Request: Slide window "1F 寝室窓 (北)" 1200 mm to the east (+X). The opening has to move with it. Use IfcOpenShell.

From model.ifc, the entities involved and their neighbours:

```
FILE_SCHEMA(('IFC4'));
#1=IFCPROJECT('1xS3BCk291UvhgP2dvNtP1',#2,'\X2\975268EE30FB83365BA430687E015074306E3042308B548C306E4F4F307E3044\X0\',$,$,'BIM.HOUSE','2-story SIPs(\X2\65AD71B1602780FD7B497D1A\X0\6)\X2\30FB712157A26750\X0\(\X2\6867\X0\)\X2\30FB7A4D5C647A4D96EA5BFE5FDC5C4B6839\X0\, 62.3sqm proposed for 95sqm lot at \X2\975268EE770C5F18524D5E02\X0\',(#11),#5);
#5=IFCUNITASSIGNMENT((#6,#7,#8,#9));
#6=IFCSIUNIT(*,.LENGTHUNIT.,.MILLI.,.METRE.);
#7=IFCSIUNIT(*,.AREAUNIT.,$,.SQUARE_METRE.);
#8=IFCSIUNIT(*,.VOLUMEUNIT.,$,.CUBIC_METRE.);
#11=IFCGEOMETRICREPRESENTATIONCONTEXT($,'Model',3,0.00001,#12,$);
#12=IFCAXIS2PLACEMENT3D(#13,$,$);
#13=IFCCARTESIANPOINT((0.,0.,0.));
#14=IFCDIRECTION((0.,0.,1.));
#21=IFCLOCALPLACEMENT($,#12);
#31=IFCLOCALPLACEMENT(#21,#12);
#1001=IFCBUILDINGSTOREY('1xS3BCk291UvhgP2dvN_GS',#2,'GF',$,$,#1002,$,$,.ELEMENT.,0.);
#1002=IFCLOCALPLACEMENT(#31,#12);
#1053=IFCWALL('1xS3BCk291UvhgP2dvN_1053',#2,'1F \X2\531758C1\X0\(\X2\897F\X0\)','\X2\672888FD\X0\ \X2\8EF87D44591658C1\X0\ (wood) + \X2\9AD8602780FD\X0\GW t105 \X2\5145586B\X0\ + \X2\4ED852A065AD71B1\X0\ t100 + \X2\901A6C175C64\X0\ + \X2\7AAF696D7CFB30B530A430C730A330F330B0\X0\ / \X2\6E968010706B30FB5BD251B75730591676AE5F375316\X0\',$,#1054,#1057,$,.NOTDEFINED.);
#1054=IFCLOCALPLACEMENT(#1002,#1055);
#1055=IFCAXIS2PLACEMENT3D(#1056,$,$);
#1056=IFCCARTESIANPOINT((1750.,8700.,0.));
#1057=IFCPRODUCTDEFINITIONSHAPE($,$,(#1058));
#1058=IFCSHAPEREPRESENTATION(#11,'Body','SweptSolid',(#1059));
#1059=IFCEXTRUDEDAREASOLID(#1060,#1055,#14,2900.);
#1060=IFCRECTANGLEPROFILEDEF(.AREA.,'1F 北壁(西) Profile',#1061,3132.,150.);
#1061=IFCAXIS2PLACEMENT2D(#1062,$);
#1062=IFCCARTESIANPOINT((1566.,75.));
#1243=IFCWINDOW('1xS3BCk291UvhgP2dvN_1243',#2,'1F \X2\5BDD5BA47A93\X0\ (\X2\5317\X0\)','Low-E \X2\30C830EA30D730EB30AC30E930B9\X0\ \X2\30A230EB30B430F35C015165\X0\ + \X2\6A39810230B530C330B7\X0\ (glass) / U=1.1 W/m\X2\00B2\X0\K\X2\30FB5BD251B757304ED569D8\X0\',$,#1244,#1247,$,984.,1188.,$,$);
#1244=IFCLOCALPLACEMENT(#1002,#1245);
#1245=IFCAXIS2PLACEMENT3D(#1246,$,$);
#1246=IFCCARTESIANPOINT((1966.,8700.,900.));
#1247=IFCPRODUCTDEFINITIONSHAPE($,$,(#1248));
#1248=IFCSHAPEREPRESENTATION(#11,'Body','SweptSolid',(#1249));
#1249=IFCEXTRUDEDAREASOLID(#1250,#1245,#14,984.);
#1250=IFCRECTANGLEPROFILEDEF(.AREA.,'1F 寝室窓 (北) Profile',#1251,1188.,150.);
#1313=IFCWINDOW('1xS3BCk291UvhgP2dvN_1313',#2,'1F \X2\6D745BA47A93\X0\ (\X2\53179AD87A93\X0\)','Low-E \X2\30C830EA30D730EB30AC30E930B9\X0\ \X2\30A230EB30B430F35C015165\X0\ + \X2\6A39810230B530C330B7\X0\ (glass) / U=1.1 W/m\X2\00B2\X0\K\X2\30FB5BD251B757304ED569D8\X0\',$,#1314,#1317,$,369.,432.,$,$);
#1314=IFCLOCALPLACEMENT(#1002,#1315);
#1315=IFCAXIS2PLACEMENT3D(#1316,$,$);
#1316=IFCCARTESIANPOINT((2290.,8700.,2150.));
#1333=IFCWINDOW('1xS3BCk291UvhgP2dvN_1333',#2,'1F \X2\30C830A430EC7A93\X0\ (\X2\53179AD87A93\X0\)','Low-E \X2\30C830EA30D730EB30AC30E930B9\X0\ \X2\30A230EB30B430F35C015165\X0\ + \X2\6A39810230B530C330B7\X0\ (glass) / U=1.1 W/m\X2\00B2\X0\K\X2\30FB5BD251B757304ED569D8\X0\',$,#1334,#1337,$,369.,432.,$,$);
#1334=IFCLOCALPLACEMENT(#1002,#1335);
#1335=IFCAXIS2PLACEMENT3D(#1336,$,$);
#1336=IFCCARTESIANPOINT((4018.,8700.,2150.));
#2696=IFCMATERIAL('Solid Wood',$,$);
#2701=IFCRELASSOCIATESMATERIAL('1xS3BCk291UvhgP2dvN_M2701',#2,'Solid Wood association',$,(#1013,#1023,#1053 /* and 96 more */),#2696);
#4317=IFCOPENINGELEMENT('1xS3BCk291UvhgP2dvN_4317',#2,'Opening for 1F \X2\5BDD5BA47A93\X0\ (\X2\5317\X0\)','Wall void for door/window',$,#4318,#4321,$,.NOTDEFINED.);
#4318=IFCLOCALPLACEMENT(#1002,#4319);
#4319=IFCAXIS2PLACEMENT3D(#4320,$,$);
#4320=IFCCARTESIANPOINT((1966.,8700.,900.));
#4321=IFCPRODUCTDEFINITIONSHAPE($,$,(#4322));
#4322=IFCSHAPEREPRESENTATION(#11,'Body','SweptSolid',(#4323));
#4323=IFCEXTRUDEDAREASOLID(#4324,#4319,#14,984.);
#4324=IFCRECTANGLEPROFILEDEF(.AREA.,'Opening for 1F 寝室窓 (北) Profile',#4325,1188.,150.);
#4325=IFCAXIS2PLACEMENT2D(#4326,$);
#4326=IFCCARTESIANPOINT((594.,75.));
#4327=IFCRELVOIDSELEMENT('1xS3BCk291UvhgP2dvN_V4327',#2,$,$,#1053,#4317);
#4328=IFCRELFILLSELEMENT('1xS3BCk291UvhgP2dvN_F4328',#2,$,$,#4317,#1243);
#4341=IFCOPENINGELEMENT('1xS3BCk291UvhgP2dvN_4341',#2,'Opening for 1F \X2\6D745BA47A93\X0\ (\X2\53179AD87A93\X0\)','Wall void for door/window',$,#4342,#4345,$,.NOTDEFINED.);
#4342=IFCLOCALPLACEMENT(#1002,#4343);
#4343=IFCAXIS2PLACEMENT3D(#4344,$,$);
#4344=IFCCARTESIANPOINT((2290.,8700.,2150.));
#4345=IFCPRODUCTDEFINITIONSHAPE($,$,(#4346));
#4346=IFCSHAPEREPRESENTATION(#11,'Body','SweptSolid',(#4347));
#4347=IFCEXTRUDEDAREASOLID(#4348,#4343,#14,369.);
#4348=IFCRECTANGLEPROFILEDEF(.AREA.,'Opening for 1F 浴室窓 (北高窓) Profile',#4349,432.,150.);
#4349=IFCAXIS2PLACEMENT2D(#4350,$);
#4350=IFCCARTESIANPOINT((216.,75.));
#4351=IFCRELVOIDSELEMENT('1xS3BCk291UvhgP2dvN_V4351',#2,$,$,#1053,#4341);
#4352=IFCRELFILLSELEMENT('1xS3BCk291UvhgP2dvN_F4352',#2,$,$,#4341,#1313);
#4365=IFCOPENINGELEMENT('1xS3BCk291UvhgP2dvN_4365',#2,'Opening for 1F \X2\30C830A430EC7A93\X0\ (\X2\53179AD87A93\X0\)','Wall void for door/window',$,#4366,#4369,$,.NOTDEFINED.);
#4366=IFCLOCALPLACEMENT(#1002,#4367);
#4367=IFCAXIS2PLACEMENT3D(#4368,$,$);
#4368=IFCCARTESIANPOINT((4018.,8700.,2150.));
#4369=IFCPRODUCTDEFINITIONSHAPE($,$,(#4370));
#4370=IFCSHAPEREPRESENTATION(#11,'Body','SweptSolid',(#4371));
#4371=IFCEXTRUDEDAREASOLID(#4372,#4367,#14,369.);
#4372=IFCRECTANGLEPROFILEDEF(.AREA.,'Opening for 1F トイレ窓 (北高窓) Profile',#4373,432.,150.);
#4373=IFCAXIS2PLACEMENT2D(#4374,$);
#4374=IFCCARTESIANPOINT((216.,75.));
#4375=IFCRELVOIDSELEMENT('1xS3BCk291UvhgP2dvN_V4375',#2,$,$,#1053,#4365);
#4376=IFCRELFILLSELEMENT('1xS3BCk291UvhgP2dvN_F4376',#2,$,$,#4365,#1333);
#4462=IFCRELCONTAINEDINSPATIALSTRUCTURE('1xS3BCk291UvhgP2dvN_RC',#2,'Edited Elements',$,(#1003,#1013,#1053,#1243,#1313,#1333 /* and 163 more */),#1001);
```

```python
import ifcopenshell
import ifcopenshell.api.geometry
import ifcopenshell.util.placement
import ifcopenshell.util.unit

model = ifcopenshell.open("model.ifc")
unit_scale = ifcopenshell.util.unit.calculate_unit_scale(model)

window = model.by_id(1243)
opening = window.FillsVoids[0].RelatingOpeningElement
wall = opening.VoidsElements[0].RelatingBuildingElement

wall_matrix = ifcopenshell.util.placement.get_local_placement(wall.ObjectPlacement)
shift = wall_matrix[:3, 0] * 1.2 / unit_scale
before = ifcopenshell.util.placement.get_local_placement(window.ObjectPlacement)[:3, 3].copy()

# The window is not placed relative to its opening, so move both.
for product in (opening, window):
    matrix = ifcopenshell.util.placement.get_local_placement(product.ObjectPlacement)
    matrix[:3, 3] += shift
    ifcopenshell.api.geometry.edit_object_placement(model, product=product, matrix=matrix, is_si=False)

after = ifcopenshell.util.placement.get_local_placement(window.ObjectPlacement)[:3, 3]
print("window moved by", (after - before).round(3) + 0.0)

model.write("model_rev.ifc")
```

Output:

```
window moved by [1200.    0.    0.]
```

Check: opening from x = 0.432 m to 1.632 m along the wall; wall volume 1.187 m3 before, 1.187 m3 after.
